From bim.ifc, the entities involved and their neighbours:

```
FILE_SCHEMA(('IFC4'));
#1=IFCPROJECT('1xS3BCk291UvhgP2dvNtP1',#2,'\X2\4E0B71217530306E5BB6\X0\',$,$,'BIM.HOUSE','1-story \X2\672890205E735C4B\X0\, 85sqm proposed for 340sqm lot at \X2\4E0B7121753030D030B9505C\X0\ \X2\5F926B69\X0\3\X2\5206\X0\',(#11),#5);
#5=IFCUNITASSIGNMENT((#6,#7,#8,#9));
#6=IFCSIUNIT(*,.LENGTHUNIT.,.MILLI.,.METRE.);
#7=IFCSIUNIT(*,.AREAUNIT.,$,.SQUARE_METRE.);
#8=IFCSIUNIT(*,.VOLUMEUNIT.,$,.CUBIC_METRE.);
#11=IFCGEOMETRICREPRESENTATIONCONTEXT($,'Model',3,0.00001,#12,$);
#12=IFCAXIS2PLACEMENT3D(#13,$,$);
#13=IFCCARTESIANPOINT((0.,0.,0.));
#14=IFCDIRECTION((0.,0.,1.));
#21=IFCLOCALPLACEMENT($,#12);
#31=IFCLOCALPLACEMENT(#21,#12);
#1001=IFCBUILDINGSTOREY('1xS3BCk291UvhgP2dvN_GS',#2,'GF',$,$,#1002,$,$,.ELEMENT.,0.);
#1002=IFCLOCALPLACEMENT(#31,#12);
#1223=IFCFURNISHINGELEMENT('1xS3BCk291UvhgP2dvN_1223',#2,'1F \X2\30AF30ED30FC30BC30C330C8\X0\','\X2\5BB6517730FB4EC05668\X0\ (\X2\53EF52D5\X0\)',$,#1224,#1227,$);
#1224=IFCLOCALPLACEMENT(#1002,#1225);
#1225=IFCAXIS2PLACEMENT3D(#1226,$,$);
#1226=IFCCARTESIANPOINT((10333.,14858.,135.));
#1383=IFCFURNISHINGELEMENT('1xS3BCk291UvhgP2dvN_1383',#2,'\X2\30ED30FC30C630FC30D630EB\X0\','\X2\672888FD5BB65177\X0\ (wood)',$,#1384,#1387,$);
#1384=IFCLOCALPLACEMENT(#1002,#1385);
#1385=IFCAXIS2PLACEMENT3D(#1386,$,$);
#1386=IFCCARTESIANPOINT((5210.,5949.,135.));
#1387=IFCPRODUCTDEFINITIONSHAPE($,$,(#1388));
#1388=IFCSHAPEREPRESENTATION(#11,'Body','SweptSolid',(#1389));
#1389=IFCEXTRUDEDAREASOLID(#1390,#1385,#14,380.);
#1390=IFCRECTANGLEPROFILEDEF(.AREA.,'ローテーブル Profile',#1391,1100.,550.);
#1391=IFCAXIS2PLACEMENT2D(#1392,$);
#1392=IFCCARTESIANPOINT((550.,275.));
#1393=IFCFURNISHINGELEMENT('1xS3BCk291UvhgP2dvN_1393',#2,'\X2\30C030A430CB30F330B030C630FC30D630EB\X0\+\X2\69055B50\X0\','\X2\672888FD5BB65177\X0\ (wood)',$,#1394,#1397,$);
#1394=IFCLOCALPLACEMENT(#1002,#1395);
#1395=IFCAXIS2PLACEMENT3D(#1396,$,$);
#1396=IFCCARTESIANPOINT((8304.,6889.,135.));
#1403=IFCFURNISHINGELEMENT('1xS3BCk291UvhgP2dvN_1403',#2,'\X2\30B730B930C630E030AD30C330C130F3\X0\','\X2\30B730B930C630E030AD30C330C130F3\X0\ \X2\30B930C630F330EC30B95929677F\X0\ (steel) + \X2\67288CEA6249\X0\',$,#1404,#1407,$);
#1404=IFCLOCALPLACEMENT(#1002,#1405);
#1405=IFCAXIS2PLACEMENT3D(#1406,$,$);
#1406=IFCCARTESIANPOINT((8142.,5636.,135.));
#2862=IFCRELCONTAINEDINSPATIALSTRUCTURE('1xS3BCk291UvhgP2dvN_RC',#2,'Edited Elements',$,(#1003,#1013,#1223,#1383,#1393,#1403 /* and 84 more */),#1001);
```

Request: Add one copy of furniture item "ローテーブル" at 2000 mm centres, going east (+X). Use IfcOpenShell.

```python
import numpy as np
import ifcopenshell
import ifcopenshell.api.geometry
import ifcopenshell.api.root
import ifcopenshell.util.element
import ifcopenshell.util.placement
import ifcopenshell.util.unit

model = ifcopenshell.open("bim.ifc")
unit_scale = ifcopenshell.util.unit.calculate_unit_scale(model)


def reuse_history(source, copy):
    """copy_class also copies each property set's owner history, people and application; keep the originals."""
    for rel in copy.IsDefinedBy:
        if rel.is_a("IfcRelDefinesByProperties") and (history := rel.RelatingPropertyDefinition.OwnerHistory):
            rel.RelatingPropertyDefinition.OwnerHistory = source.OwnerHistory
            ifcopenshell.util.element.remove_deep2(model, history)


source = model.by_id(1383)
base = ifcopenshell.util.placement.get_local_placement(source.ObjectPlacement)
step = np.array([1.0, 0.0, 0.0]) * 2 / unit_scale

for i in range(1, 2):
    copy = ifcopenshell.api.root.copy_class(model, product=source)
    copy.Representation = ifcopenshell.util.element.copy_deep(
        model, source.Representation, exclude=["IfcGeometricRepresentationContext", "IfcRepresentationMap"]
    )
    reuse_history(source, copy)
    matrix = base.copy()
    matrix[:3, 3] += i * step
    print("added at", matrix[:3, 3].round(3) + 0.0)
    ifcopenshell.api.geometry.edit_object_placement(model, product=copy, matrix=matrix, is_si=False)

model.write("bim_updated.ifc")
```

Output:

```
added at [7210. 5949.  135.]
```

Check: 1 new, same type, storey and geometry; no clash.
